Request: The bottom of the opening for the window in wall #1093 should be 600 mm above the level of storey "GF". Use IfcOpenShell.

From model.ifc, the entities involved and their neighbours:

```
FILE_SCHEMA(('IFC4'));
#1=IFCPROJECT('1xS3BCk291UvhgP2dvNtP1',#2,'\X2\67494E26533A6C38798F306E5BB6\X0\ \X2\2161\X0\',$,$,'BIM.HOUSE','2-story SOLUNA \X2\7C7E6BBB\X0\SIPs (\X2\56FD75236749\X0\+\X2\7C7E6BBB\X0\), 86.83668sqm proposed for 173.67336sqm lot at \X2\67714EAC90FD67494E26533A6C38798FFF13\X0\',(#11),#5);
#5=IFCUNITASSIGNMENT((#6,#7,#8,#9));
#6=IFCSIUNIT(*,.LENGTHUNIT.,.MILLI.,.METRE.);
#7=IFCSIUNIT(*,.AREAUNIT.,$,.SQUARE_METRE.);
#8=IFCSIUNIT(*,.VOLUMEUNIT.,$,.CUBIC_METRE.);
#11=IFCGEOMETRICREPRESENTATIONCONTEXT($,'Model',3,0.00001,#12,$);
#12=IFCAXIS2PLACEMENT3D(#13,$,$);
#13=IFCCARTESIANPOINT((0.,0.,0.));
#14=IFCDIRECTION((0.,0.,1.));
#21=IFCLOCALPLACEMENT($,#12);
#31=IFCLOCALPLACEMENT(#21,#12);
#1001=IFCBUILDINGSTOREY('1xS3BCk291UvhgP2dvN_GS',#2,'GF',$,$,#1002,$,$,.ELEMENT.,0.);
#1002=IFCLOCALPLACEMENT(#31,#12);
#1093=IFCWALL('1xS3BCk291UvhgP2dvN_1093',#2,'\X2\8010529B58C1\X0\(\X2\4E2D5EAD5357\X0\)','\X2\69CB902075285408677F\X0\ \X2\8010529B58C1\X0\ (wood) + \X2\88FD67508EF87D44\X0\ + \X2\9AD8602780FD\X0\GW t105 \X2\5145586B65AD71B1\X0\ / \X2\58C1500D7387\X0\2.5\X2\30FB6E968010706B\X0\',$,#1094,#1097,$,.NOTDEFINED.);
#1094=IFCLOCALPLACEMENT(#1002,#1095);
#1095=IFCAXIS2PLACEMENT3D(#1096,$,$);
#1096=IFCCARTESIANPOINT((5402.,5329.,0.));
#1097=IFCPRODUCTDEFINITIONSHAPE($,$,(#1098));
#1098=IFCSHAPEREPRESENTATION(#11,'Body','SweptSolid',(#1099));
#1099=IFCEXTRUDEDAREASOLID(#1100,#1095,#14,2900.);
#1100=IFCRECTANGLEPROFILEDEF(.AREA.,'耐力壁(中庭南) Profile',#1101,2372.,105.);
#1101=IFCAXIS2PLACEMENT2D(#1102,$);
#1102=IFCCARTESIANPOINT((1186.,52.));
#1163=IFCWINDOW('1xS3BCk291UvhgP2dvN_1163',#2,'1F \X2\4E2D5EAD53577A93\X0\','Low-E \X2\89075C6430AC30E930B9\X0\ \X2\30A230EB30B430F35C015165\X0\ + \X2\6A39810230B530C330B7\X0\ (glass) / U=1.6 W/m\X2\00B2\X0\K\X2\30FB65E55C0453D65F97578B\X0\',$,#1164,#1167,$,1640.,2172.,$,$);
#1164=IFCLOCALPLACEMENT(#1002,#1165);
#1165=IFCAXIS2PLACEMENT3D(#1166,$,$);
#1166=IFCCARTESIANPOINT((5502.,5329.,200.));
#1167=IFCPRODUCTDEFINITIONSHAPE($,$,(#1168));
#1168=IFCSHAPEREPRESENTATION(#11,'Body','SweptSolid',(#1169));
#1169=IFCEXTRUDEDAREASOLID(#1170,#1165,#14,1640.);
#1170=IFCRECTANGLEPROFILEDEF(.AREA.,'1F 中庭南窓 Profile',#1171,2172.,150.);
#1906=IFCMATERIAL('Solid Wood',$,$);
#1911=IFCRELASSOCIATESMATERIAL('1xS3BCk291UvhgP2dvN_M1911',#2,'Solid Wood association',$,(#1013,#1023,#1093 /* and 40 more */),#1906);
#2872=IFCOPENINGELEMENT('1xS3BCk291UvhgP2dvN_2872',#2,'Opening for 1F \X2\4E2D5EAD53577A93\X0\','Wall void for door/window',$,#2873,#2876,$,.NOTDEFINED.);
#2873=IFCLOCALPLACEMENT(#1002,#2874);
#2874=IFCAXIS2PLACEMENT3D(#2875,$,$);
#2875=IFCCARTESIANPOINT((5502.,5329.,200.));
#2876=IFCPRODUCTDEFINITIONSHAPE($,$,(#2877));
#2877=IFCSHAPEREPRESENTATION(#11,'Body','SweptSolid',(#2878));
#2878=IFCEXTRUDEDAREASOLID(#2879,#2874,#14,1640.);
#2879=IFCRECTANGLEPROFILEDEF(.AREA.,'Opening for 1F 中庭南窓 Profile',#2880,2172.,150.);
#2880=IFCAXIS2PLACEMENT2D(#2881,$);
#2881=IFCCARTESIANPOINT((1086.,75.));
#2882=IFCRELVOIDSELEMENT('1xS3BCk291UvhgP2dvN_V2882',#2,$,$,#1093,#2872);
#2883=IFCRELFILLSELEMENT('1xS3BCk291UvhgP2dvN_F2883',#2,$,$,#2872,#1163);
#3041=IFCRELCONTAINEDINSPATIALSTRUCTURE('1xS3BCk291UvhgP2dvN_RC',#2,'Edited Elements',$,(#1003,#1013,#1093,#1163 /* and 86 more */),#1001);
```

```python
import numpy as np
import ifcopenshell
import ifcopenshell.api.geometry
import ifcopenshell.geom
import ifcopenshell.util.element
import ifcopenshell.util.placement
import ifcopenshell.util.shape
import ifcopenshell.util.unit

model = ifcopenshell.open("model.ifc")
unit_scale = ifcopenshell.util.unit.calculate_unit_scale(model)

window = model.by_id(1163)
opening = window.FillsVoids[0].RelatingOpeningElement
storey = ifcopenshell.util.element.get_container(window, ifc_class="IfcBuildingStorey")
level = ifcopenshell.util.placement.get_local_placement(storey.ObjectPlacement)[2, 3]

# The opening's origin need not be at the sill, so measure its lowest point.
shape = ifcopenshell.geom.create_shape(ifcopenshell.geom.settings(), opening)
bottom = ifcopenshell.util.shape.get_shape_bottom_elevation(shape, shape.geometry) / unit_scale
dz = level + 0.6 / unit_scale - bottom

shift = np.array([0.0, 0.0, dz])
# The window is not placed relative to its opening, so move both.
for product in (opening, window):
    matrix = ifcopenshell.util.placement.get_local_placement(product.ObjectPlacement)
    matrix[:3, 3] += shift
    ifcopenshell.api.geometry.edit_object_placement(model, product=product, matrix=matrix, is_si=False)

print(f"moved by {dz * unit_scale:+.3f} m")

model.write("model_v2.ifc")
```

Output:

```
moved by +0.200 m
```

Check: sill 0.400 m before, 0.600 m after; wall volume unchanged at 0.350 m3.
